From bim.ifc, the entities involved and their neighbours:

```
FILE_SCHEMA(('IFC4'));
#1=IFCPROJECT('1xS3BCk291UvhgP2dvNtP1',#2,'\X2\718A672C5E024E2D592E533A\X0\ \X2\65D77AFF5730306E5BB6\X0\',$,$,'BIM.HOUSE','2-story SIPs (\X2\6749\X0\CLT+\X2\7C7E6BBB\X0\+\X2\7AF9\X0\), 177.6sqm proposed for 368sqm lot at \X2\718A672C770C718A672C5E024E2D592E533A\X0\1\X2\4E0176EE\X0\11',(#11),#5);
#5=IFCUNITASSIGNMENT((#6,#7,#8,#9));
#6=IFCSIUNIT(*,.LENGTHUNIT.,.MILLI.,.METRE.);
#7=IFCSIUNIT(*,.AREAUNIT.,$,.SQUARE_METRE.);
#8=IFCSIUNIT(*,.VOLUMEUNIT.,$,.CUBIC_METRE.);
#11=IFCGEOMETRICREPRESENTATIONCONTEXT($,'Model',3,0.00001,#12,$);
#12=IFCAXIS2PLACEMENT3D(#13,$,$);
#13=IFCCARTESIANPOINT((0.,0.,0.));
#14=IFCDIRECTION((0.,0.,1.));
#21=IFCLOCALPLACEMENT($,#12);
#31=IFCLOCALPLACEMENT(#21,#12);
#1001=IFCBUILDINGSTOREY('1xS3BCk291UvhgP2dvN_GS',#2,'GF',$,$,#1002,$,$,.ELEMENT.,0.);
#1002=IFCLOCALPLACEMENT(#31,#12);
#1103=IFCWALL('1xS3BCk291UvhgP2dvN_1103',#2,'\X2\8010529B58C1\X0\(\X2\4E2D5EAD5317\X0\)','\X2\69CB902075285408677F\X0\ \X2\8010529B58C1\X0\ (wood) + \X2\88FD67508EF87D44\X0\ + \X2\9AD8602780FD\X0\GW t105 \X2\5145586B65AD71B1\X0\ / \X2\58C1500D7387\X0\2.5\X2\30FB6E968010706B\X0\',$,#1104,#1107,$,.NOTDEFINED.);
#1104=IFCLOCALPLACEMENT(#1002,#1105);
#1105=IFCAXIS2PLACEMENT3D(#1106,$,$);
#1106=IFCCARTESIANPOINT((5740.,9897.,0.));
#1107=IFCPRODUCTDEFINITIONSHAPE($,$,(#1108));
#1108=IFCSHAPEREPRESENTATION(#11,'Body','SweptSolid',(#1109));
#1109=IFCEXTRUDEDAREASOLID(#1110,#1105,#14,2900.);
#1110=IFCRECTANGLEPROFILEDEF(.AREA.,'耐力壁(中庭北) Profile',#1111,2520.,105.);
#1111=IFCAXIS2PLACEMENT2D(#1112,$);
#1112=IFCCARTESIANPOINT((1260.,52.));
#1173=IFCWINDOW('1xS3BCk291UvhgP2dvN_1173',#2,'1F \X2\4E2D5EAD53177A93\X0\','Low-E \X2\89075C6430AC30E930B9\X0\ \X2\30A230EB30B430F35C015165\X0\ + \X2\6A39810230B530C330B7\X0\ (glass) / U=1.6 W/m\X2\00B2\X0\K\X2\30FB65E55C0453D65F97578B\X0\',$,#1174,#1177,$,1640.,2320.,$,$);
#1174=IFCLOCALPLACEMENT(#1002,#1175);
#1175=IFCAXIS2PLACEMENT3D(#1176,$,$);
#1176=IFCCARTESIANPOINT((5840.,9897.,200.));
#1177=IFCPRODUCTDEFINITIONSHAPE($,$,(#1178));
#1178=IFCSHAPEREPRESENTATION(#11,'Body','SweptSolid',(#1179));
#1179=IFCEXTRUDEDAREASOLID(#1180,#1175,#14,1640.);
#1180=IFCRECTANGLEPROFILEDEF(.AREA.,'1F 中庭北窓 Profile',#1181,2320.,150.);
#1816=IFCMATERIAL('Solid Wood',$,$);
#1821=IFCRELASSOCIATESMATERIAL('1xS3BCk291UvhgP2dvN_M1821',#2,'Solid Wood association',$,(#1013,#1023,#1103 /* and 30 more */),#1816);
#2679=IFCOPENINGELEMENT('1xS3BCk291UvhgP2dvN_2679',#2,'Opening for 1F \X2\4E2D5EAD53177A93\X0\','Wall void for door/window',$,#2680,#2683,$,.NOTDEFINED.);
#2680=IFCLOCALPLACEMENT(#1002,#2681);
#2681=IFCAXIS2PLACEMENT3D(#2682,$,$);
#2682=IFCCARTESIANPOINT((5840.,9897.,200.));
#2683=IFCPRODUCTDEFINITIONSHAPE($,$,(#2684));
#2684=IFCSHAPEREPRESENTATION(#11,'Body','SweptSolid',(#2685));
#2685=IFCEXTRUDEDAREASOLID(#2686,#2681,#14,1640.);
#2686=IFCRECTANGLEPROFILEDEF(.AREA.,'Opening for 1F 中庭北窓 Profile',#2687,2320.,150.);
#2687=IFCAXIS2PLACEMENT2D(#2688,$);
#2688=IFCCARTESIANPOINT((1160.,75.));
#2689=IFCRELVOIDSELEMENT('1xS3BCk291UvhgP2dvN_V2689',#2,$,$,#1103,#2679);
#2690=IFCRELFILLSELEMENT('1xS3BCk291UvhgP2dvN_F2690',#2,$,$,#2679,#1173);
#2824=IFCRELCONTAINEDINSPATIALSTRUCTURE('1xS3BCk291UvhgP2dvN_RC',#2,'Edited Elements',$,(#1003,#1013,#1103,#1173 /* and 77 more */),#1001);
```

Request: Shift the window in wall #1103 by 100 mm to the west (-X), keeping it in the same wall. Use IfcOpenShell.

```python
import ifcopenshell
import ifcopenshell.api.geometry
import ifcopenshell.util.placement

model = ifcopenshell.open("bim.ifc")

window = model.by_guid("1xS3BCk291UvhgP2dvN_1173")
opening = window.FillsVoids[0].RelatingOpeningElement
wall = opening.VoidsElements[0].RelatingBuildingElement

wall_matrix = ifcopenshell.util.placement.get_local_placement(wall.ObjectPlacement)
shift = wall_matrix[:3, 0] * -100.0
before = ifcopenshell.util.placement.get_local_placement(window.ObjectPlacement)[:3, 3].copy()

# The window is not placed relative to its opening, so move both.
for product in (opening, window):
    matrix = ifcopenshell.util.placement.get_local_placement(product.ObjectPlacement)
    matrix[:3, 3] += shift
    ifcopenshell.api.geometry.edit_object_placement(model, product=product, matrix=matrix, is_si=False)

after = ifcopenshell.util.placement.get_local_placement(window.ObjectPlacement)[:3, 3]
print("window moved by", (after - before).round(3) + 0.0)

model.write("bim_updated.ifc")
```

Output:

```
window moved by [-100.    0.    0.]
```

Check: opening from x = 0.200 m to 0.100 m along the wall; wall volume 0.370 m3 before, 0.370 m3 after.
